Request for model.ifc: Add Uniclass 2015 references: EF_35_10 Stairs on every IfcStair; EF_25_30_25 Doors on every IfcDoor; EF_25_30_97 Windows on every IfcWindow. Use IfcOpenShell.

First a look at what the model holds.

```python
import ifcopenshell

model = ifcopenshell.open("model.ifc")
print(model.schema)
print("classifications:", [c.Name for c in model.by_type("IfcClassification")])
for ifc_class in ("IfcDoor", "IfcRoof", "IfcStair", "IfcWall", "IfcWindow"):
    print(ifc_class, len(model.by_type(ifc_class)))
```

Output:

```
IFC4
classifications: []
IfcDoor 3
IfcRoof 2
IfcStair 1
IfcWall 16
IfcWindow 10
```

```python
import ifcopenshell
import ifcopenshell.api.classification

model = ifcopenshell.open("model.ifc")

system = ifcopenshell.api.classification.add_classification(model, classification="Uniclass 2015")

codes = {
    "IfcStair": ("EF_35_10", "Stairs"),
    "IfcDoor": ("EF_25_30_25", "Doors"),
    "IfcWindow": ("EF_25_30_97", "Windows"),
}
for ifc_class, (code, name) in codes.items():
    products = model.by_type(ifc_class)
    ifcopenshell.api.classification.add_reference(
        model, products=products, classification=system, identification=code, name=name
    )
    print(code, len(products))

model.write("model_rev.ifc")
```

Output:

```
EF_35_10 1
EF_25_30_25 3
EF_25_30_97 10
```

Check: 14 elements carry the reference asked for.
